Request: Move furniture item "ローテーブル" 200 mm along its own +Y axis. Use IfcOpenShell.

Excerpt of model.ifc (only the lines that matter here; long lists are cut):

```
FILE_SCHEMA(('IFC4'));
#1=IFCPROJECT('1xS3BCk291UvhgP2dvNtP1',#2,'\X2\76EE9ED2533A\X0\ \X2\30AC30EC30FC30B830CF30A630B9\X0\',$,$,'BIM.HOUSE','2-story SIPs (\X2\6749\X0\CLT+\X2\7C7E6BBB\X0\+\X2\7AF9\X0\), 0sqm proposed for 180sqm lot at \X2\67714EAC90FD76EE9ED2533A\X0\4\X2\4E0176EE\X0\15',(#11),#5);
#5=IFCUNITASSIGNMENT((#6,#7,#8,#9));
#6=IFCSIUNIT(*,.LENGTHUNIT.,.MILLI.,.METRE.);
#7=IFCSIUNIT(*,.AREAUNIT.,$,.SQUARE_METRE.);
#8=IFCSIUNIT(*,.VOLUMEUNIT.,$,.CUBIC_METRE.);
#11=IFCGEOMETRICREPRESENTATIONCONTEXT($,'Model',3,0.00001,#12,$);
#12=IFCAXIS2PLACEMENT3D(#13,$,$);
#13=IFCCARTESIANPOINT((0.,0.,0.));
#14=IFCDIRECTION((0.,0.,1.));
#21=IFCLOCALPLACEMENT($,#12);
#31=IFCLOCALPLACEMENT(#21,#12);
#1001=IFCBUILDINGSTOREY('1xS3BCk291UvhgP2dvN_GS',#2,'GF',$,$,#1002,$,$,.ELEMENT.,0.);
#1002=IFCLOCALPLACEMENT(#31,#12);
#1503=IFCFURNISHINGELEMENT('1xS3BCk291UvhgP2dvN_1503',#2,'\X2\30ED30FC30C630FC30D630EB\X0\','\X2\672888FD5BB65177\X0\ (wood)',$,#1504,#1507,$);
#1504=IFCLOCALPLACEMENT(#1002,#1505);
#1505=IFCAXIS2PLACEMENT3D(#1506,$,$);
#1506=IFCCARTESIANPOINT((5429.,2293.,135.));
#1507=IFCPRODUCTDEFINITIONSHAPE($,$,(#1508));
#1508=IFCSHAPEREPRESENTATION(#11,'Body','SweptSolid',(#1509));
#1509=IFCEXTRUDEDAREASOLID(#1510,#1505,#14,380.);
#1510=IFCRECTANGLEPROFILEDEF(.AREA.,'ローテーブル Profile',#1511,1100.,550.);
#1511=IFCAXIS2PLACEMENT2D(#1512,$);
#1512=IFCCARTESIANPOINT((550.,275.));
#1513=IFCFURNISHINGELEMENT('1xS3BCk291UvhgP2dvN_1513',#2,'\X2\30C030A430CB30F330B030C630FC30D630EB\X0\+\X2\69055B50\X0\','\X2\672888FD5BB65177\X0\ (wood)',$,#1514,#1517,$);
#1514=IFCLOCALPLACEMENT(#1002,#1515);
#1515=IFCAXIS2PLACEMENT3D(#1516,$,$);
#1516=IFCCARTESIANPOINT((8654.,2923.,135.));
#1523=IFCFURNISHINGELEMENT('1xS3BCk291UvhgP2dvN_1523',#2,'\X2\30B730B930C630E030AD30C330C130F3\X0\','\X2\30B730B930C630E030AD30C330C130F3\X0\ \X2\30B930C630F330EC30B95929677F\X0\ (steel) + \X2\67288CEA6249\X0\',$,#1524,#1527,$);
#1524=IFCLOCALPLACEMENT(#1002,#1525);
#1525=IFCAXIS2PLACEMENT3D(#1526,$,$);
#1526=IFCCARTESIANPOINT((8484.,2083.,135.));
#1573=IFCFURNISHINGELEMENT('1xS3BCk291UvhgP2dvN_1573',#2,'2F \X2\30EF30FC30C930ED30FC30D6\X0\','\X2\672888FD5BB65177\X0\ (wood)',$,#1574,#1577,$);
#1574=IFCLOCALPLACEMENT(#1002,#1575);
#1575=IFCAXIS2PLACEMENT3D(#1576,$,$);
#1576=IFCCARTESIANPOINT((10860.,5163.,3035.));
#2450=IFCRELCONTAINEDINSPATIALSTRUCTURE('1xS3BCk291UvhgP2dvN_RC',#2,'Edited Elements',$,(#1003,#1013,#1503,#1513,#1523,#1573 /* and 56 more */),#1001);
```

```python
import ifcopenshell
import ifcopenshell.api.geometry
import ifcopenshell.util.placement
import ifcopenshell.util.unit

model = ifcopenshell.open("model.ifc")
unit_scale = ifcopenshell.util.unit.calculate_unit_scale(model)

item = model.by_guid("1xS3BCk291UvhgP2dvN_1503")
matrix = ifcopenshell.util.placement.get_local_placement(item.ObjectPlacement)
matrix[:3, 3] += matrix[:3, 1] * 0.2 / unit_scale
ifcopenshell.api.geometry.edit_object_placement(model, product=item, matrix=matrix, is_si=False)

print(ifcopenshell.util.placement.get_local_placement(item.ObjectPlacement).round(3) + 0.0)

model.write("model_rev.ifc")
```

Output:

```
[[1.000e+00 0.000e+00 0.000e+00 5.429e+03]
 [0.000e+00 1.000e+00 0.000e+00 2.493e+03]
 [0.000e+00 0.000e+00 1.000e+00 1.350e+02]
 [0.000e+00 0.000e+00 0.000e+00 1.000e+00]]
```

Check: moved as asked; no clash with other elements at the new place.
